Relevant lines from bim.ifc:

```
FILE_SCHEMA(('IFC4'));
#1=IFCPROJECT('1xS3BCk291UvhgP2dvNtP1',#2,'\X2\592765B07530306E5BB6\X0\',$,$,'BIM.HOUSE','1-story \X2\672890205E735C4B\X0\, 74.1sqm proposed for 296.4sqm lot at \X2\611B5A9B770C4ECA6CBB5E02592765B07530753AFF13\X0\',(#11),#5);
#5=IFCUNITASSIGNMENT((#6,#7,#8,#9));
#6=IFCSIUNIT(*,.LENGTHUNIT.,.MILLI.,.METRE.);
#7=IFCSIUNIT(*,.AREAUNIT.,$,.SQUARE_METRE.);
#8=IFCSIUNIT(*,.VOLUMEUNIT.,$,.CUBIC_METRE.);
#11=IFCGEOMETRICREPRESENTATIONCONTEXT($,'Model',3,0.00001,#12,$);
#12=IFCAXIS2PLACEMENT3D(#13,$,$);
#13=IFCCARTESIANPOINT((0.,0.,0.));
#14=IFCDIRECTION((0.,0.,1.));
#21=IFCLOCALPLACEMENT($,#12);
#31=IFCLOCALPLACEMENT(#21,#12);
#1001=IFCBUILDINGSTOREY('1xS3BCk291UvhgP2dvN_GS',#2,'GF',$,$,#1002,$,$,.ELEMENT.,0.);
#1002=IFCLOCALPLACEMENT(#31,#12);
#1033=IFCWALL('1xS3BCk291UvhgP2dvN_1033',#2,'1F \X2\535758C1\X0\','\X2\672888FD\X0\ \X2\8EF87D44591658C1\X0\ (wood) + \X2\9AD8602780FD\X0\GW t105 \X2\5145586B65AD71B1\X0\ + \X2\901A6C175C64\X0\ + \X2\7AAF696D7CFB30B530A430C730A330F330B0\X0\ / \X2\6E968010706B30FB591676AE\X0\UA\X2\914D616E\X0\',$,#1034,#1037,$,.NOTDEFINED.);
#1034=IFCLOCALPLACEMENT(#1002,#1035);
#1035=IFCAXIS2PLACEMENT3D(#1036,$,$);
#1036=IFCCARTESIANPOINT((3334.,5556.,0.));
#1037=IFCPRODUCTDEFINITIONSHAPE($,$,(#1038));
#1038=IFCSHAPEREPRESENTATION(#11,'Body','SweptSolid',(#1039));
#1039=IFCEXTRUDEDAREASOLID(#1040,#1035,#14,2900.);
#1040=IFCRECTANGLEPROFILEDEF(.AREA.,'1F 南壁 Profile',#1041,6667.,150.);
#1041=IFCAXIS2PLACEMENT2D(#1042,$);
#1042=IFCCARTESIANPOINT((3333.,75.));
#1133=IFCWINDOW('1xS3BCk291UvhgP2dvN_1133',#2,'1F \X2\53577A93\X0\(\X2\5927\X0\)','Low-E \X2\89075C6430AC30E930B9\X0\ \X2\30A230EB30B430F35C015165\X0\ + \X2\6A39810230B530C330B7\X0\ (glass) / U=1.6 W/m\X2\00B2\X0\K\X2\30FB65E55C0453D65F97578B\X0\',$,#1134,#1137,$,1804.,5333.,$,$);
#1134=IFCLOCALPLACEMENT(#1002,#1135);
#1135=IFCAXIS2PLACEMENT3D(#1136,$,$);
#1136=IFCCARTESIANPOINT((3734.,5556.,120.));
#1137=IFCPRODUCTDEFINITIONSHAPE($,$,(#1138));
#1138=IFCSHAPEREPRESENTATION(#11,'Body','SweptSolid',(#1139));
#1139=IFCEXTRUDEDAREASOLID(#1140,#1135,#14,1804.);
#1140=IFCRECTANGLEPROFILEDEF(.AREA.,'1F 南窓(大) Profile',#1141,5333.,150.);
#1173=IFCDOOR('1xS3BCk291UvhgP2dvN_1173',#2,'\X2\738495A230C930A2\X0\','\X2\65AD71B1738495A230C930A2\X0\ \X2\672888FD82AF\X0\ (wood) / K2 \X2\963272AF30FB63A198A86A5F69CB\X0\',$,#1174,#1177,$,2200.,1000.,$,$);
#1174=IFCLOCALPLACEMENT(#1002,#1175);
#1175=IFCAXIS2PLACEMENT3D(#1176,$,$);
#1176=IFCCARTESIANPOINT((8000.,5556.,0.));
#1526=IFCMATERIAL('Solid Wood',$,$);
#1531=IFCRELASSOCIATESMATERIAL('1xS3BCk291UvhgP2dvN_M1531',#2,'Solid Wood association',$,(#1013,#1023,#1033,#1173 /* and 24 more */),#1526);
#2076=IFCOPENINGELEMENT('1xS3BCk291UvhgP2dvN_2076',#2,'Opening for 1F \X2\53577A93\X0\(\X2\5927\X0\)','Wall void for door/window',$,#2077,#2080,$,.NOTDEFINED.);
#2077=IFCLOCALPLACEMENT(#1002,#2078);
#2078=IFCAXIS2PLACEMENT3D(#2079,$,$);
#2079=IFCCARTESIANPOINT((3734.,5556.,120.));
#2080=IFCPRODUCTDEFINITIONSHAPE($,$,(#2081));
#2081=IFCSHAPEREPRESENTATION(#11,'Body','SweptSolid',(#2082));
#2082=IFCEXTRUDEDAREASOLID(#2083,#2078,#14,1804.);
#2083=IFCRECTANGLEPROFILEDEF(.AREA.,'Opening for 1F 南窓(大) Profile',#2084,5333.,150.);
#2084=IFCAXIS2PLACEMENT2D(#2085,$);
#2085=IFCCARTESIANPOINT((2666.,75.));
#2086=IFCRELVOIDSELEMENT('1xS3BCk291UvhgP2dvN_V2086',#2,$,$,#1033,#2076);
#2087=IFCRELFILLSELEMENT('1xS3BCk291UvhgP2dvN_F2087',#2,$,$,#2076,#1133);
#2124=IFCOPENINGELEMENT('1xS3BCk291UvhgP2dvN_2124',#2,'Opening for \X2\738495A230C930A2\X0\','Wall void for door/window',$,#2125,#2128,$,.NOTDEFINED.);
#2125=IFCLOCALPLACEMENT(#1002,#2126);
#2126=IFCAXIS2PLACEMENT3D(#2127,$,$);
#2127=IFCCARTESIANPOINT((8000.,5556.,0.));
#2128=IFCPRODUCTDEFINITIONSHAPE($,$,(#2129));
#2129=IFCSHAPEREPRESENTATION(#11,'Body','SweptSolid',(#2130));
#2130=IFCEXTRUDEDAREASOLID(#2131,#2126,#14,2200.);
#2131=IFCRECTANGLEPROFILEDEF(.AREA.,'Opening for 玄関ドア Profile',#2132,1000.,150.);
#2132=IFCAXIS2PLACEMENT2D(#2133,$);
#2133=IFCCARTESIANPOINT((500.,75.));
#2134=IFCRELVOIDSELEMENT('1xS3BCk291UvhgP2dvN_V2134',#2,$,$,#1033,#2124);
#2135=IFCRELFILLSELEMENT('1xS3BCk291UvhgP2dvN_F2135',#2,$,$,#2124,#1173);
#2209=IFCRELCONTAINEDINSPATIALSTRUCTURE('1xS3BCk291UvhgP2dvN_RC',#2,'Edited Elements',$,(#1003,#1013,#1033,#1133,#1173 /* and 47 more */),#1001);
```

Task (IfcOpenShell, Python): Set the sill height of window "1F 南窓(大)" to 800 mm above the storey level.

```python
import numpy as np
import ifcopenshell
import ifcopenshell.api.geometry
import ifcopenshell.geom
import ifcopenshell.util.element
import ifcopenshell.util.placement
import ifcopenshell.util.shape
import ifcopenshell.util.unit

model = ifcopenshell.open("bim.ifc")
unit_scale = ifcopenshell.util.unit.calculate_unit_scale(model)

window = model.by_guid("1xS3BCk291UvhgP2dvN_1133")
opening = window.FillsVoids[0].RelatingOpeningElement
storey = ifcopenshell.util.element.get_container(window, ifc_class="IfcBuildingStorey")
level = ifcopenshell.util.placement.get_local_placement(storey.ObjectPlacement)[2, 3]

# The opening's origin need not be at the sill, so measure its lowest point.
shape = ifcopenshell.geom.create_shape(ifcopenshell.geom.settings(), opening)
bottom = ifcopenshell.util.shape.get_shape_bottom_elevation(shape, shape.geometry) / unit_scale
dz = level + 0.8 / unit_scale - bottom

shift = np.array([0.0, 0.0, dz])
# The window is not placed relative to its opening, so move both.
for product in (opening, window):
    matrix = ifcopenshell.util.placement.get_local_placement(product.ObjectPlacement)
    matrix[:3, 3] += shift
    ifcopenshell.api.geometry.edit_object_placement(model, product=product, matrix=matrix, is_si=False)

print(f"moved by {dz * unit_scale:+.3f} m")

model.write("bim_rev.ifc")
```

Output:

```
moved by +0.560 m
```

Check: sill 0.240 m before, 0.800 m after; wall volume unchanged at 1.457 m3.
